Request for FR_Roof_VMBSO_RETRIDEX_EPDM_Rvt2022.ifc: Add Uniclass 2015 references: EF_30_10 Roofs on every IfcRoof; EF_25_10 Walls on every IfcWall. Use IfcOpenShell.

First a look at what the model holds.

```python
import ifcopenshell

model = ifcopenshell.open("FR_Roof_VMBSO_RETRIDEX_EPDM_Rvt2022.ifc")
print(model.schema)
print("classifications:", [c.Name for c in model.by_type("IfcClassification")])
for ifc_class in ("IfcDoor", "IfcRoof", "IfcStair", "IfcWall", "IfcWindow"):
    print(ifc_class, len(model.by_type(ifc_class)))
```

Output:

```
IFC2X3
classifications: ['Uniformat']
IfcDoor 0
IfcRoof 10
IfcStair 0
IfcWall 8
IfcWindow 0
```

```python
import ifcopenshell
import ifcopenshell.api.classification

model = ifcopenshell.open("FR_Roof_VMBSO_RETRIDEX_EPDM_Rvt2022.ifc")

# IFC2X3 requires Source and Edition and has no link from the project to the system.
system = model.create_entity("IfcClassification", Source="NBS", Edition="2015", Name="Uniclass 2015")

codes = {
    "IfcRoof": ("EF_30_10", "Roofs"),
    "IfcWall": ("EF_25_10", "Walls"),
}
for ifc_class, (code, name) in codes.items():
    products = model.by_type(ifc_class)
    ifcopenshell.api.classification.add_reference(
        model, products=products, classification=system, identification=code, name=name
    )
    print(code, len(products))

model.write("FR_Roof_VMBSO_RETRIDEX_EPDM_Rvt2022_v2.ifc")
```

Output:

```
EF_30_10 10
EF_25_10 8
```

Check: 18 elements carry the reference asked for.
